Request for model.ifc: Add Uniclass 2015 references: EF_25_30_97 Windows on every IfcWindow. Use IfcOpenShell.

First a look at what the model holds.

```python
import ifcopenshell

model = ifcopenshell.open("model.ifc")
print(model.schema)
print("classifications:", [c.Name for c in model.by_type("IfcClassification")])
for ifc_class in ("IfcDoor", "IfcRoof", "IfcStair", "IfcWall", "IfcWindow"):
    print(ifc_class, len(model.by_type(ifc_class)))
```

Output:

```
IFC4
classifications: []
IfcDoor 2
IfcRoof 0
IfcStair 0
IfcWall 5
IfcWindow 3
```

```python
import ifcopenshell
import ifcopenshell.api.classification

model = ifcopenshell.open("model.ifc")

system = ifcopenshell.api.classification.add_classification(model, classification="Uniclass 2015")

codes = {
    "IfcWindow": ("EF_25_30_97", "Windows"),
}
for ifc_class, (code, name) in codes.items():
    products = model.by_type(ifc_class)
    ifcopenshell.api.classification.add_reference(
        model, products=products, classification=system, identification=code, name=name
    )
    print(code, len(products))

model.write("model_edited.ifc")
```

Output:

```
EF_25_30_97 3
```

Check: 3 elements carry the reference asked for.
